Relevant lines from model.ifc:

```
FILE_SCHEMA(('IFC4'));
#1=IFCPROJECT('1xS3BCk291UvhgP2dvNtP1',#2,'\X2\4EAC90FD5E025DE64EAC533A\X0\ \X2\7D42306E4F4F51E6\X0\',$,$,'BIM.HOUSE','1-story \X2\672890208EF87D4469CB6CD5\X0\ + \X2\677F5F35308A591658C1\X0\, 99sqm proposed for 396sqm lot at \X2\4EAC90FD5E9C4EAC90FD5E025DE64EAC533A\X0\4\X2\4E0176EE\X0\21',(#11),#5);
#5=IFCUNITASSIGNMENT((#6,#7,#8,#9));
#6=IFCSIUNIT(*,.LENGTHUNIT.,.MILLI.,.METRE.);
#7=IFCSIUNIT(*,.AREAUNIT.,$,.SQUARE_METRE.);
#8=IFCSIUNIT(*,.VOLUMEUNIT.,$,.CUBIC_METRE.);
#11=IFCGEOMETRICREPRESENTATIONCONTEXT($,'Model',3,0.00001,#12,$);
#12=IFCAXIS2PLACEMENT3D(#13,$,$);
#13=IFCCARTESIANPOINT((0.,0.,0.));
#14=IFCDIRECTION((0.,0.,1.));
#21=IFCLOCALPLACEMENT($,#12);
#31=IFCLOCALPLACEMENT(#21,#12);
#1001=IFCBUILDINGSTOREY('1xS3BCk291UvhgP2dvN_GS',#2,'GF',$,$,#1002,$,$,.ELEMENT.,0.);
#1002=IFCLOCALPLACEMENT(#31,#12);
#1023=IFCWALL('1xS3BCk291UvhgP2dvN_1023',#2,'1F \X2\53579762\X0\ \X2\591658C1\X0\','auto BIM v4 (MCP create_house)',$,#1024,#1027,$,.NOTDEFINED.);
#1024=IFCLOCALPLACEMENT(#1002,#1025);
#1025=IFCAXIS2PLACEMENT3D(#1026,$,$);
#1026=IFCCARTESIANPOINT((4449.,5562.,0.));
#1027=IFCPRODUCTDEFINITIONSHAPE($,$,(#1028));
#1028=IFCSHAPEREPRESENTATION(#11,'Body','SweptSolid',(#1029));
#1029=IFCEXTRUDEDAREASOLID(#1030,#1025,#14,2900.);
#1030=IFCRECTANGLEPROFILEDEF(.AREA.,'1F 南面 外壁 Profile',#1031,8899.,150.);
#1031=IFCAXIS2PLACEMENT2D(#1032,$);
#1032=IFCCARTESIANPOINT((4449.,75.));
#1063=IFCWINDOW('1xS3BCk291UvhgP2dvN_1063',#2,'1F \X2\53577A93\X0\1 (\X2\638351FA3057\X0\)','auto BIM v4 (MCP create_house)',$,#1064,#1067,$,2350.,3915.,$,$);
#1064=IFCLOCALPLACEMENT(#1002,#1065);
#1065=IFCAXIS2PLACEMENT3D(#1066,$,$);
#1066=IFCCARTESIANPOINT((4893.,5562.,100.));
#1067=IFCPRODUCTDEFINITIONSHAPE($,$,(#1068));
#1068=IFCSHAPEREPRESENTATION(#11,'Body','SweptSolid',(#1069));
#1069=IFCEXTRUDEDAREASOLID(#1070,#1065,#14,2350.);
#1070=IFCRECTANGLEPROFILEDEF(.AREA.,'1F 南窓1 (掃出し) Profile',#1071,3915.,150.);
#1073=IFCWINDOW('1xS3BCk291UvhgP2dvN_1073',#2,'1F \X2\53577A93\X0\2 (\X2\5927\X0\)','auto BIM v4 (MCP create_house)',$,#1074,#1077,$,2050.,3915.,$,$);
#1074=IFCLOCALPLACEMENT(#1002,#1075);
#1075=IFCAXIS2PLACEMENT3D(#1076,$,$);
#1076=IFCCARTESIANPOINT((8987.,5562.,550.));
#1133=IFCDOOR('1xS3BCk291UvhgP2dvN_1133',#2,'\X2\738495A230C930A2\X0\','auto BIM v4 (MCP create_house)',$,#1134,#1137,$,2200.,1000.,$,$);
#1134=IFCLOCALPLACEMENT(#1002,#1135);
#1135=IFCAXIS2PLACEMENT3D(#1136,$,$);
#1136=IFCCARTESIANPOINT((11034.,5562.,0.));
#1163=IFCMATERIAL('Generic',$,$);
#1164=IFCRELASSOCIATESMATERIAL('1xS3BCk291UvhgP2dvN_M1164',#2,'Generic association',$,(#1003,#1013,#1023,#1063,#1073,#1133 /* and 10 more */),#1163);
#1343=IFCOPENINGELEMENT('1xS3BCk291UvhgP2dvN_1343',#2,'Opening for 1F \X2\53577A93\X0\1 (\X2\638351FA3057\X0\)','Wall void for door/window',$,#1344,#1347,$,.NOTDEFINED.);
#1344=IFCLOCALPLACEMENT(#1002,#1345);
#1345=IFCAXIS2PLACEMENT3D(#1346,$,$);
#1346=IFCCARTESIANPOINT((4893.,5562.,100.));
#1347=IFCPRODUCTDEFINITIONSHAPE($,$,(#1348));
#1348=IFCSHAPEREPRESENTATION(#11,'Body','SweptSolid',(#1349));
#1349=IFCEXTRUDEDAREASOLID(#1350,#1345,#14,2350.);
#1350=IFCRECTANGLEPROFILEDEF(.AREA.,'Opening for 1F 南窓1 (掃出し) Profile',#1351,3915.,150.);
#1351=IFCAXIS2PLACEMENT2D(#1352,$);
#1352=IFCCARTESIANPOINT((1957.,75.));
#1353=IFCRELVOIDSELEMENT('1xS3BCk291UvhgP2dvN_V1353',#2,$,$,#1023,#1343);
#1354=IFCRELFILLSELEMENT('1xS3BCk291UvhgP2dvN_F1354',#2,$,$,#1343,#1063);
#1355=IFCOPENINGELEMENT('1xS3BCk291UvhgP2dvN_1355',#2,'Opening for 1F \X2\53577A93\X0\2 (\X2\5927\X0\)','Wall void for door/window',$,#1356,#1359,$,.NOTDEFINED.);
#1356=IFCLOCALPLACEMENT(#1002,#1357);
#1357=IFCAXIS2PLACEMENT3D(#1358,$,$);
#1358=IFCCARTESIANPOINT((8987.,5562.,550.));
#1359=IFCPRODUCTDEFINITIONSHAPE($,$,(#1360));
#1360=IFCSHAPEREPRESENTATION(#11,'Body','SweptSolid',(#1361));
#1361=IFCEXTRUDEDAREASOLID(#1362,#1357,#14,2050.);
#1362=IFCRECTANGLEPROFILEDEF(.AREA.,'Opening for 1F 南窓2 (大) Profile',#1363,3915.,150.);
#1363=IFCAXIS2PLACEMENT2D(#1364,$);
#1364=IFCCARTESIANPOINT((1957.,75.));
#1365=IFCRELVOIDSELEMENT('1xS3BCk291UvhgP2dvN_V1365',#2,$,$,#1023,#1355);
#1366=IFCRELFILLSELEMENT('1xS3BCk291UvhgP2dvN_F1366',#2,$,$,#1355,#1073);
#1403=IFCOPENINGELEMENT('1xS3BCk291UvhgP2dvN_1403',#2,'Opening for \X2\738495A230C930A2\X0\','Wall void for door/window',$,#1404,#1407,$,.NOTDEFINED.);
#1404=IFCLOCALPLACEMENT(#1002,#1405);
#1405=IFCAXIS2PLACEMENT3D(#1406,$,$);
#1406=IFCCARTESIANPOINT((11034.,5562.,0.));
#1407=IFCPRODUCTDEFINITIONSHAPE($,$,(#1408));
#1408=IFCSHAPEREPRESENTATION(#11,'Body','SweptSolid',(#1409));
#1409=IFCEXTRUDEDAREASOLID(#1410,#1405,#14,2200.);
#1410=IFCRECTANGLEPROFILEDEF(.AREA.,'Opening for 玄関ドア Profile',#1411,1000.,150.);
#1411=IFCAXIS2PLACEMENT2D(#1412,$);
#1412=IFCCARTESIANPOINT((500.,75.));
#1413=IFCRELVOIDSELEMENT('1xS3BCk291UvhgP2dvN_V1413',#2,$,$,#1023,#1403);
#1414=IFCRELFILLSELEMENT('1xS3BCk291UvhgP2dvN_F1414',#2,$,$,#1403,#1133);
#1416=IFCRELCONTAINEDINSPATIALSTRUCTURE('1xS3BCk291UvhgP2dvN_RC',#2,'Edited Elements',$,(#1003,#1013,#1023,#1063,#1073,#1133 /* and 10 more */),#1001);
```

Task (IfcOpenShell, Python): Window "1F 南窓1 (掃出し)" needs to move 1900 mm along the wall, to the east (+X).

```python
import ifcopenshell
import ifcopenshell.api.geometry
import ifcopenshell.util.placement

model = ifcopenshell.open("model.ifc")

window = model.by_guid("1xS3BCk291UvhgP2dvN_1063")
opening = window.FillsVoids[0].RelatingOpeningElement
wall = opening.VoidsElements[0].RelatingBuildingElement

wall_matrix = ifcopenshell.util.placement.get_local_placement(wall.ObjectPlacement)
shift = wall_matrix[:3, 0] * 1900.0
before = ifcopenshell.util.placement.get_local_placement(window.ObjectPlacement)[:3, 3].copy()

# The window is not placed relative to its opening, so move both.
for product in (opening, window):
    matrix = ifcopenshell.util.placement.get_local_placement(product.ObjectPlacement)
    matrix[:3, 3] += shift
    ifcopenshell.api.geometry.edit_object_placement(model, product=product, matrix=matrix, is_si=False)

after = ifcopenshell.util.placement.get_local_placement(window.ObjectPlacement)[:3, 3]
print("window moved by", (after - before).round(3) + 0.0)

model.write("model_updated.ifc")
```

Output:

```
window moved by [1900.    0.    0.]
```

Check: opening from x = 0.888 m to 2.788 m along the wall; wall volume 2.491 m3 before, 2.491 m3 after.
